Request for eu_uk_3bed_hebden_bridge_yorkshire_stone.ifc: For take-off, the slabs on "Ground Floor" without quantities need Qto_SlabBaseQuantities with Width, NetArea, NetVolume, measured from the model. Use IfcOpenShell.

First a look at what the model holds.

```python
import ifcopenshell
import ifcopenshell.util.element
import ifcopenshell.util.unit

model = ifcopenshell.open("eu_uk_3bed_hebden_bridge_yorkshire_stone.ifc")
print(model.schema)
for unit_type in ("LENGTHUNIT", "AREAUNIT", "VOLUMEUNIT"):
    print(unit_type, ifcopenshell.util.unit.calculate_unit_scale(model, unit_type))
storey = next(s for s in model.by_type("IfcBuildingStorey") if s.Name == "Ground Floor")
slabs = [e for e in ifcopenshell.util.element.get_decomposition(storey) if e.is_a("IfcSlab")]
for e in sorted(slabs, key=lambda e: e.id()):
    print(e.id(), e.is_a(), e.Name, list(ifcopenshell.util.element.get_psets(e, qtos_only=True)), sep=" | ")
```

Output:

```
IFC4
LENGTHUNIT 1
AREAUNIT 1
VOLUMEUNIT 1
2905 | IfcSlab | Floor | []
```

```python
import ifcopenshell
import ifcopenshell.api.pset
import ifcopenshell.geom
import ifcopenshell.util.element
import ifcopenshell.util.shape
import ifcopenshell.util.unit

model = ifcopenshell.open("eu_uk_3bed_hebden_bridge_yorkshire_stone.ifc")
unit_scale = ifcopenshell.util.unit.calculate_unit_scale(model)
area_scale = ifcopenshell.util.unit.calculate_unit_scale(model, "AREAUNIT")
volume_scale = ifcopenshell.util.unit.calculate_unit_scale(model, "VOLUMEUNIT")
settings = ifcopenshell.geom.settings()

storey = next(s for s in model.by_type("IfcBuildingStorey") if s.Name == "Ground Floor")
slabs = [e for e in ifcopenshell.util.element.get_decomposition(storey) if e.is_a("IfcSlab")]

for e in sorted(slabs, key=lambda e: e.id()):
    if ifcopenshell.util.element.get_psets(e, qtos_only=True, should_inherit=False):
        continue
    # Geometry comes back in metres, in the element's own axes.
    shape = ifcopenshell.geom.create_shape(settings, e)
    values = {
        "Width": ifcopenshell.util.shape.get_z(shape.geometry) / unit_scale,
        "NetArea": ifcopenshell.util.shape.get_footprint_area(shape.geometry) / area_scale,
        "NetVolume": ifcopenshell.util.shape.get_volume(shape.geometry) / volume_scale,
    }
    qto = ifcopenshell.api.pset.add_qto(model, product=e, name="Qto_SlabBaseQuantities")
    ifcopenshell.api.pset.edit_qto(model, qto=qto, properties=values)
    print(e.id(), {k: round(v, 3) for k, v in values.items()})

model.write("eu_uk_3bed_hebden_bridge_yorkshire_stone_updated.ifc")
```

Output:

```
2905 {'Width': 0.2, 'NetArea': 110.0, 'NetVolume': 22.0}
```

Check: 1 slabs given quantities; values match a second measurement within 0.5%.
